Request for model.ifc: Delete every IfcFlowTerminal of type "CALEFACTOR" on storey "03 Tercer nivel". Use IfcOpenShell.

First a look at what the model holds.

```python
import ifcopenshell
import ifcopenshell.util.element

model = ifcopenshell.open("model.ifc")
print(model.schema)
storey = next(s for s in model.by_type("IfcBuildingStorey") if s.Name == "03 Tercer nivel")
terminals = [e for e in ifcopenshell.util.element.get_decomposition(storey) if e.is_a("IfcFlowTerminal")]
seen = {}
for e in terminals:
    element_type = ifcopenshell.util.element.get_type(e)
    name = element_type.Name if element_type not in (None, e) else None
    seen[name] = seen.get(name, 0) + 1
for name, count in sorted(seen.items(), key=str):
    print(count, "x", name)
```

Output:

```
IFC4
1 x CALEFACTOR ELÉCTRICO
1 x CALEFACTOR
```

```python
import ifcopenshell
import ifcopenshell.api.root
import ifcopenshell.util.element

model = ifcopenshell.open("model.ifc")

storey = next(s for s in model.by_type("IfcBuildingStorey") if s.Name == "03 Tercer nivel")
terminals = [e for e in ifcopenshell.util.element.get_decomposition(storey) if e.is_a("IfcFlowTerminal")]
targets = [e for e in terminals if (t := ifcopenshell.util.element.get_type(e)) not in (None, e) and t.Name == "CALEFACTOR"]

for e in targets:
    ifcopenshell.api.root.remove_product(model, product=e)
print(len(targets), "removed")

model.write("model_rev.ifc")
```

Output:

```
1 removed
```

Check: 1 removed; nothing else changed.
